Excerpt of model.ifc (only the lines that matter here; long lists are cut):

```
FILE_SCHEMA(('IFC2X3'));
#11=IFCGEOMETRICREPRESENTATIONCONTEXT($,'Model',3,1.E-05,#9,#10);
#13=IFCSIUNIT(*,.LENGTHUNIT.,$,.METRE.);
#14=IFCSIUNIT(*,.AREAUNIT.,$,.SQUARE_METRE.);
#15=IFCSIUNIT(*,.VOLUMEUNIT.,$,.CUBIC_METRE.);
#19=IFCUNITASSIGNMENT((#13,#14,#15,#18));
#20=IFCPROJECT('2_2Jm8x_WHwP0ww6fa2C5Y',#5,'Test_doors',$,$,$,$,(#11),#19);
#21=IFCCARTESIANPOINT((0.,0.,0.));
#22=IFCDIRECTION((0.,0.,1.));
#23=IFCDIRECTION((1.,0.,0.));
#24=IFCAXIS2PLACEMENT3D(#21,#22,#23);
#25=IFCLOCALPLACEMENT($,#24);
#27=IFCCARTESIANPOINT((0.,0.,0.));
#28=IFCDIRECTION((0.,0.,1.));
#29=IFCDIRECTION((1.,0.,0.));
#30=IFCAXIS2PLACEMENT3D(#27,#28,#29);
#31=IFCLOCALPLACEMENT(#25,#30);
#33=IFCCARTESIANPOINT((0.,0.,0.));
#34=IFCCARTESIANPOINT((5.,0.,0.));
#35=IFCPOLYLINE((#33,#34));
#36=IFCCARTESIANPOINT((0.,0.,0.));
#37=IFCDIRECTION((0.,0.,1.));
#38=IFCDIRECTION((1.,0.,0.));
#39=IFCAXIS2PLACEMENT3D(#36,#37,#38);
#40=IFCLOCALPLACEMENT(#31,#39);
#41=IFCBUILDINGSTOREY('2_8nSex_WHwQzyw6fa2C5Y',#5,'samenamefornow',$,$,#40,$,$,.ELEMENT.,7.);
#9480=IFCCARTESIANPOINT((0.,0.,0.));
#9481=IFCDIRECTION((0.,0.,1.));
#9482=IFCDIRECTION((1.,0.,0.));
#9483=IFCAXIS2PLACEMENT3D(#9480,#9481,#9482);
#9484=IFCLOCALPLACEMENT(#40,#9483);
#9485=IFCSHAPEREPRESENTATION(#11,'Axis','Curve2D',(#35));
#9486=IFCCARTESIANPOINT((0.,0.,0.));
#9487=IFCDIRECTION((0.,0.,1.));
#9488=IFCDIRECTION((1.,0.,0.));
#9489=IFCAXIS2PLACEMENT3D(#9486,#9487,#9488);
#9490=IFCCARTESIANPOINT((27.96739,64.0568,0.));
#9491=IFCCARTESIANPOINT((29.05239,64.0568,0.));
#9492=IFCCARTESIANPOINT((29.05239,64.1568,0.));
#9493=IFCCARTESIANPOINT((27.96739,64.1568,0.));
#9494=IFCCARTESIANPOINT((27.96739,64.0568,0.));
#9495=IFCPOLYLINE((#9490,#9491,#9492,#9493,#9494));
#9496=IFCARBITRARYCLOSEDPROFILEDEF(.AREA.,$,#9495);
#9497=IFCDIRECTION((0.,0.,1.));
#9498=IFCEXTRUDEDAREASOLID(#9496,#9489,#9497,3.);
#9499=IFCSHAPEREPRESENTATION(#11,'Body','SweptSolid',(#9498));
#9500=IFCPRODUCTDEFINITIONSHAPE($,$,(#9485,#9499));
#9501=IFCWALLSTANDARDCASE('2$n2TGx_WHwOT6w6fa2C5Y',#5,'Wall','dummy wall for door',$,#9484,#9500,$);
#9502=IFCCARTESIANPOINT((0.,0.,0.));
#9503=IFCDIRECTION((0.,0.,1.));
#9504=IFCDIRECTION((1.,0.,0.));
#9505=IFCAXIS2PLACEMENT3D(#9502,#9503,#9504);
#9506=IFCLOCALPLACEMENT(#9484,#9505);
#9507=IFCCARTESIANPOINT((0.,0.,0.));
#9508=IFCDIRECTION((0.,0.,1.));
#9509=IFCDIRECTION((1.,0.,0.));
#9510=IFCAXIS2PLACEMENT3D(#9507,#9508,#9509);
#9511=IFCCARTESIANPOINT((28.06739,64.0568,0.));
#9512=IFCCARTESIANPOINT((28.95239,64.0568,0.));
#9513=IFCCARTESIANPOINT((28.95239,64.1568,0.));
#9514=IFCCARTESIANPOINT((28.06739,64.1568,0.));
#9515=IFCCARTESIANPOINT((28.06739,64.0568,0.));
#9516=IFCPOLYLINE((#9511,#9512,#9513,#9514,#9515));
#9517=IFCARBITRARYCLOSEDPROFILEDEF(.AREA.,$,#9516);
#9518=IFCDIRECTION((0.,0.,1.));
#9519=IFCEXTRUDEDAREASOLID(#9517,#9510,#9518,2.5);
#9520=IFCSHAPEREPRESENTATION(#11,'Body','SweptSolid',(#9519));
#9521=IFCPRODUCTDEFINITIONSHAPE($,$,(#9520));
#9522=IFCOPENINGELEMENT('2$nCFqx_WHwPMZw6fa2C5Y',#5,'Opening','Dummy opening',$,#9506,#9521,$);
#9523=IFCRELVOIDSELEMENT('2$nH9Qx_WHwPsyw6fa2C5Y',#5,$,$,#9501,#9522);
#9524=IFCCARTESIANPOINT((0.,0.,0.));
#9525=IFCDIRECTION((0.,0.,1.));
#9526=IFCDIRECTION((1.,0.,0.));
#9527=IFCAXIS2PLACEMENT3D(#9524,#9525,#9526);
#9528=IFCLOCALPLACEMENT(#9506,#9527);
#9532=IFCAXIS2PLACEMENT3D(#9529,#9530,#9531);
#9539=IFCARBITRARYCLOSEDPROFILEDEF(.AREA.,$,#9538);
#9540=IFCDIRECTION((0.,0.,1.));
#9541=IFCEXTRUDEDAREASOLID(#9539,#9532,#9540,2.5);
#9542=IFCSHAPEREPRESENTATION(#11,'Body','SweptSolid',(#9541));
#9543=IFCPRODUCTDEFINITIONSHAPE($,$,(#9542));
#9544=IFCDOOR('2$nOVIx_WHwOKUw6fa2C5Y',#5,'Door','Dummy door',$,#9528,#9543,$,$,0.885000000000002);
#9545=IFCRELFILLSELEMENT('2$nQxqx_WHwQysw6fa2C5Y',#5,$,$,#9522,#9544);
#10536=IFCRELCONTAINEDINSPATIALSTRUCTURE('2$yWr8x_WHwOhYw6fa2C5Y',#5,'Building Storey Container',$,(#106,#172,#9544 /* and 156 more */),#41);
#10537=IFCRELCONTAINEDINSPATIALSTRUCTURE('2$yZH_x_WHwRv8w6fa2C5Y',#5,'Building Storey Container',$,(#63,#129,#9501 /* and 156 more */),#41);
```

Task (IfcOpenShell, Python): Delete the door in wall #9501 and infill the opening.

```python
import ifcopenshell
import ifcopenshell.api.feature
import ifcopenshell.api.root
import ifcopenshell.geom
import ifcopenshell.util.shape

model = ifcopenshell.open("model.ifc")
settings = ifcopenshell.geom.settings()


def volume(element):
    """Net volume in cubic metres, openings subtracted."""
    shape = ifcopenshell.geom.create_shape(settings, element)
    return ifcopenshell.util.shape.get_volume(shape.geometry)


door = model.by_guid("2$nOVIx_WHwOKUw6fa2C5Y")
opening = door.FillsVoids[0].RelatingOpeningElement
wall = opening.VoidsElements[0].RelatingBuildingElement
before = volume(wall)

ifcopenshell.api.root.remove_product(model, product=door)
ifcopenshell.api.feature.remove_feature(model, feature=opening)

after = volume(wall)

print(f"wall volume {before:.3f} -> {after:.3f} m3")

model.write("model_edited.ifc")
```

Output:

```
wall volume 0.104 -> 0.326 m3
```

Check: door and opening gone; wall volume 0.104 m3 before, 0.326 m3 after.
